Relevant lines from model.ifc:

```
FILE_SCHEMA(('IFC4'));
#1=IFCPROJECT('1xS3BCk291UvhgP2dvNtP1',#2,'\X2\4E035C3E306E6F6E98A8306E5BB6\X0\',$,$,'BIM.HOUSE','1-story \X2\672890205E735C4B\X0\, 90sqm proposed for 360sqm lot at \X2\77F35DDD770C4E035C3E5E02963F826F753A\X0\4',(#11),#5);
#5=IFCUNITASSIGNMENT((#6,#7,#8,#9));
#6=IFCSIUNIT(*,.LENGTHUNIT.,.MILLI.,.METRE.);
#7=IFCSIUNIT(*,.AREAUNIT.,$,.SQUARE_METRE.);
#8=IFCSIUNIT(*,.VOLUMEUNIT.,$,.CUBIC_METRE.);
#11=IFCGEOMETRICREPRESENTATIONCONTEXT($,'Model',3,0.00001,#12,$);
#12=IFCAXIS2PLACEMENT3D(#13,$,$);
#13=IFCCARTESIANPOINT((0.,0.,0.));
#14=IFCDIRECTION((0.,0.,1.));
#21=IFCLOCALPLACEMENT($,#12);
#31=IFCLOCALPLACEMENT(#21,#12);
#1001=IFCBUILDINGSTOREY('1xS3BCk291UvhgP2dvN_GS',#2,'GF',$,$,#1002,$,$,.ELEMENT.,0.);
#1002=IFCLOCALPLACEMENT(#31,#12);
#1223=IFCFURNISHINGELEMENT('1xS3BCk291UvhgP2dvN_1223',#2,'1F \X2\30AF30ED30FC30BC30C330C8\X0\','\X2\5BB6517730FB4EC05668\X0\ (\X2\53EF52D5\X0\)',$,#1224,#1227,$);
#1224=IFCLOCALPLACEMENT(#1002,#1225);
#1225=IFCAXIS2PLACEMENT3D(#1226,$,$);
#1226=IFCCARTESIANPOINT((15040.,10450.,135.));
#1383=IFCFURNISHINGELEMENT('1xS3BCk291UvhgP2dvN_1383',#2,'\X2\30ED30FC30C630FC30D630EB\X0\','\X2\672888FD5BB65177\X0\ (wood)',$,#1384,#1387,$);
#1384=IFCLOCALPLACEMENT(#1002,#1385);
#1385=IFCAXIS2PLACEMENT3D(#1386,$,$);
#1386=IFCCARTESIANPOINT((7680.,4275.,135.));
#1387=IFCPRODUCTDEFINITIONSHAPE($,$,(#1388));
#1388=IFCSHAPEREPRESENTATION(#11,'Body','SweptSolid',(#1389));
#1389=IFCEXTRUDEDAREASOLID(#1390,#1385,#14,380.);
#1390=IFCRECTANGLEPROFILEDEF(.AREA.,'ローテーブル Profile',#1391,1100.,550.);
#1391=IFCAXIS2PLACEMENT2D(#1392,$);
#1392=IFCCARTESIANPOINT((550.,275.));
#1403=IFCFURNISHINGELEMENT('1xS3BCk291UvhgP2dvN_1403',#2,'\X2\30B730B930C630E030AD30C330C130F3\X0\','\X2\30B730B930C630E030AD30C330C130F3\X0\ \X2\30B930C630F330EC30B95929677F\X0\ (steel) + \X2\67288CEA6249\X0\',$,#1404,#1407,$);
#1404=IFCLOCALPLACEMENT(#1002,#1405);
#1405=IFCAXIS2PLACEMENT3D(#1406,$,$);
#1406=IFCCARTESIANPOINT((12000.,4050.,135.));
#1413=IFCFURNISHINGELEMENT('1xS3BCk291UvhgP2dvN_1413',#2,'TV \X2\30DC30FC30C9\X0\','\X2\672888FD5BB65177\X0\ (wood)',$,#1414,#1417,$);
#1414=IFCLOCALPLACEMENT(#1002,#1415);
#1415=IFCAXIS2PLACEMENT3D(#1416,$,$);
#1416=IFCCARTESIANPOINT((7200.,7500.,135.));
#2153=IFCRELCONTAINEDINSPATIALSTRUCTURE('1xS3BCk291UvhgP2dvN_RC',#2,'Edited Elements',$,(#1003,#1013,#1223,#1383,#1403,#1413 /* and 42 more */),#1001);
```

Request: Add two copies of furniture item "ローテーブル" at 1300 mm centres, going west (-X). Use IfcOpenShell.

```python
import numpy as np
import ifcopenshell
import ifcopenshell.api.geometry
import ifcopenshell.api.root
import ifcopenshell.util.element
import ifcopenshell.util.placement

model = ifcopenshell.open("model.ifc")


def reuse_history(source, copy):
    """copy_class also copies each property set's owner history, people and application; keep the originals."""
    for rel in copy.IsDefinedBy:
        if rel.is_a("IfcRelDefinesByProperties") and (history := rel.RelatingPropertyDefinition.OwnerHistory):
            rel.RelatingPropertyDefinition.OwnerHistory = source.OwnerHistory
            ifcopenshell.util.element.remove_deep2(model, history)


source = model.by_id(1383)
base = ifcopenshell.util.placement.get_local_placement(source.ObjectPlacement)
step = np.array([-1.0, 0.0, 0.0]) * 1300.0

for i in range(1, 3):
    copy = ifcopenshell.api.root.copy_class(model, product=source)
    copy.Representation = ifcopenshell.util.element.copy_deep(
        model, source.Representation, exclude=["IfcGeometricRepresentationContext", "IfcRepresentationMap"]
    )
    reuse_history(source, copy)
    matrix = base.copy()
    matrix[:3, 3] += i * step
    print("added at", matrix[:3, 3].round(3) + 0.0)
    ifcopenshell.api.geometry.edit_object_placement(model, product=copy, matrix=matrix, is_si=False)

model.write("model_v2.ifc")
```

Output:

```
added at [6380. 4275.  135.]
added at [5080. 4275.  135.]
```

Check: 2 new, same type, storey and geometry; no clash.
